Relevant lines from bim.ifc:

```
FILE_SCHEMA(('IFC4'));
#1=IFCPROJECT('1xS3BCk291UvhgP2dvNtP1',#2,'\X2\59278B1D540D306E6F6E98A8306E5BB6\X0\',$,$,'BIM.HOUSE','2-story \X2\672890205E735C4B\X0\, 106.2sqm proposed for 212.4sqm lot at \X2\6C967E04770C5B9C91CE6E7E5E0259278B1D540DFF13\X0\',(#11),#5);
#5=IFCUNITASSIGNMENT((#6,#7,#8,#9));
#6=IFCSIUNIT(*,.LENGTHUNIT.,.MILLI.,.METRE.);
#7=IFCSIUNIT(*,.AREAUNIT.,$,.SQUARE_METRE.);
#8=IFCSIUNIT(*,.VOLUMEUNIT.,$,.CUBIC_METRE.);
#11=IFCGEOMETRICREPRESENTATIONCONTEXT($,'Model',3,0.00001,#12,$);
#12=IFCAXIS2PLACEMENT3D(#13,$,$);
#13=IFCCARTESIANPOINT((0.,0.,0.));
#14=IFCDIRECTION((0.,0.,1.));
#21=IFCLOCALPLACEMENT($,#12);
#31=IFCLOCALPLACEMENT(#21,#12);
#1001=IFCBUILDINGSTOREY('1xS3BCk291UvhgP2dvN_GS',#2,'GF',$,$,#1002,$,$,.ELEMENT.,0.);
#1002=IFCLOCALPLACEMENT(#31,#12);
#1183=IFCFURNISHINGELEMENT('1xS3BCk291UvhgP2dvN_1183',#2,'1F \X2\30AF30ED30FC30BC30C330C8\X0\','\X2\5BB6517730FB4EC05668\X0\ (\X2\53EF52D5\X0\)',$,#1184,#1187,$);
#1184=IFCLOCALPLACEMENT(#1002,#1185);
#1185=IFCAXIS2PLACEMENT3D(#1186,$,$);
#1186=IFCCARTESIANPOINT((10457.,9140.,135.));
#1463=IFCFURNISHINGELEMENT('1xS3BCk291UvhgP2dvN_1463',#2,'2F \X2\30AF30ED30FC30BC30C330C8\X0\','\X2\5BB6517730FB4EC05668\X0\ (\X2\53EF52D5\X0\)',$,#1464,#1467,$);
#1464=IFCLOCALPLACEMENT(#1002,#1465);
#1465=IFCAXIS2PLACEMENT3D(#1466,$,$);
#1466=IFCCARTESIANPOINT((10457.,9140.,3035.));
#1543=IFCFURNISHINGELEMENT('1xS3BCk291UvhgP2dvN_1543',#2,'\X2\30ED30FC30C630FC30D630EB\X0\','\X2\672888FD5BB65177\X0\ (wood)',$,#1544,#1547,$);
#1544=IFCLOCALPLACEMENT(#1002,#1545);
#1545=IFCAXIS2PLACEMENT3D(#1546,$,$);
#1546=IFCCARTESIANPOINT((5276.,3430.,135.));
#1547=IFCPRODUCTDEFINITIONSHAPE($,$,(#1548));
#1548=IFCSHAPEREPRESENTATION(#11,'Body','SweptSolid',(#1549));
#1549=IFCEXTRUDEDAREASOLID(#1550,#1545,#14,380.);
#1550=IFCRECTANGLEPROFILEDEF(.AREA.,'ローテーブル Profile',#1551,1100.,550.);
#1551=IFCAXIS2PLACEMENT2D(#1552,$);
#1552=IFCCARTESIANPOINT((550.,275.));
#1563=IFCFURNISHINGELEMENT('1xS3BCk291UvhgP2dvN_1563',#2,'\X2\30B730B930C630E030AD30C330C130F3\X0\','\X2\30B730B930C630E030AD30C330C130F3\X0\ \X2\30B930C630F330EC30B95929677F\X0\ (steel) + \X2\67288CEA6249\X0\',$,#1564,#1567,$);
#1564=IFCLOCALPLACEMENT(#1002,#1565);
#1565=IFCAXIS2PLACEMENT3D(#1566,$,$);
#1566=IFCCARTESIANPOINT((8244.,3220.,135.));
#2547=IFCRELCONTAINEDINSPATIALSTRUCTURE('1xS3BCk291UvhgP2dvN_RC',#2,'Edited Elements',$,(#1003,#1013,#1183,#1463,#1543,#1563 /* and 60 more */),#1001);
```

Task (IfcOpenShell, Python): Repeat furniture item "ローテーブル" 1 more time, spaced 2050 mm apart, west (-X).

```python
import numpy as np
import ifcopenshell
import ifcopenshell.api.geometry
import ifcopenshell.api.root
import ifcopenshell.util.element
import ifcopenshell.util.placement
import ifcopenshell.util.unit

model = ifcopenshell.open("bim.ifc")
unit_scale = ifcopenshell.util.unit.calculate_unit_scale(model)


def reuse_history(source, copy):
    """copy_class also copies each property set's owner history, people and application; keep the originals."""
    for rel in copy.IsDefinedBy:
        if rel.is_a("IfcRelDefinesByProperties") and (history := rel.RelatingPropertyDefinition.OwnerHistory):
            rel.RelatingPropertyDefinition.OwnerHistory = source.OwnerHistory
            ifcopenshell.util.element.remove_deep2(model, history)


source = model.by_id(1543)
base = ifcopenshell.util.placement.get_local_placement(source.ObjectPlacement)
step = np.array([-1.0, 0.0, 0.0]) * 2.05 / unit_scale

for i in range(1, 2):
    copy = ifcopenshell.api.root.copy_class(model, product=source)
    copy.Representation = ifcopenshell.util.element.copy_deep(
        model, source.Representation, exclude=["IfcGeometricRepresentationContext", "IfcRepresentationMap"]
    )
    reuse_history(source, copy)
    matrix = base.copy()
    matrix[:3, 3] += i * step
    print("added at", matrix[:3, 3].round(3) + 0.0)
    ifcopenshell.api.geometry.edit_object_placement(model, product=copy, matrix=matrix, is_si=False)

model.write("bim_rev.ifc")
```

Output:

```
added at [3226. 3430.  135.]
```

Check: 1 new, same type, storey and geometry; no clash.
